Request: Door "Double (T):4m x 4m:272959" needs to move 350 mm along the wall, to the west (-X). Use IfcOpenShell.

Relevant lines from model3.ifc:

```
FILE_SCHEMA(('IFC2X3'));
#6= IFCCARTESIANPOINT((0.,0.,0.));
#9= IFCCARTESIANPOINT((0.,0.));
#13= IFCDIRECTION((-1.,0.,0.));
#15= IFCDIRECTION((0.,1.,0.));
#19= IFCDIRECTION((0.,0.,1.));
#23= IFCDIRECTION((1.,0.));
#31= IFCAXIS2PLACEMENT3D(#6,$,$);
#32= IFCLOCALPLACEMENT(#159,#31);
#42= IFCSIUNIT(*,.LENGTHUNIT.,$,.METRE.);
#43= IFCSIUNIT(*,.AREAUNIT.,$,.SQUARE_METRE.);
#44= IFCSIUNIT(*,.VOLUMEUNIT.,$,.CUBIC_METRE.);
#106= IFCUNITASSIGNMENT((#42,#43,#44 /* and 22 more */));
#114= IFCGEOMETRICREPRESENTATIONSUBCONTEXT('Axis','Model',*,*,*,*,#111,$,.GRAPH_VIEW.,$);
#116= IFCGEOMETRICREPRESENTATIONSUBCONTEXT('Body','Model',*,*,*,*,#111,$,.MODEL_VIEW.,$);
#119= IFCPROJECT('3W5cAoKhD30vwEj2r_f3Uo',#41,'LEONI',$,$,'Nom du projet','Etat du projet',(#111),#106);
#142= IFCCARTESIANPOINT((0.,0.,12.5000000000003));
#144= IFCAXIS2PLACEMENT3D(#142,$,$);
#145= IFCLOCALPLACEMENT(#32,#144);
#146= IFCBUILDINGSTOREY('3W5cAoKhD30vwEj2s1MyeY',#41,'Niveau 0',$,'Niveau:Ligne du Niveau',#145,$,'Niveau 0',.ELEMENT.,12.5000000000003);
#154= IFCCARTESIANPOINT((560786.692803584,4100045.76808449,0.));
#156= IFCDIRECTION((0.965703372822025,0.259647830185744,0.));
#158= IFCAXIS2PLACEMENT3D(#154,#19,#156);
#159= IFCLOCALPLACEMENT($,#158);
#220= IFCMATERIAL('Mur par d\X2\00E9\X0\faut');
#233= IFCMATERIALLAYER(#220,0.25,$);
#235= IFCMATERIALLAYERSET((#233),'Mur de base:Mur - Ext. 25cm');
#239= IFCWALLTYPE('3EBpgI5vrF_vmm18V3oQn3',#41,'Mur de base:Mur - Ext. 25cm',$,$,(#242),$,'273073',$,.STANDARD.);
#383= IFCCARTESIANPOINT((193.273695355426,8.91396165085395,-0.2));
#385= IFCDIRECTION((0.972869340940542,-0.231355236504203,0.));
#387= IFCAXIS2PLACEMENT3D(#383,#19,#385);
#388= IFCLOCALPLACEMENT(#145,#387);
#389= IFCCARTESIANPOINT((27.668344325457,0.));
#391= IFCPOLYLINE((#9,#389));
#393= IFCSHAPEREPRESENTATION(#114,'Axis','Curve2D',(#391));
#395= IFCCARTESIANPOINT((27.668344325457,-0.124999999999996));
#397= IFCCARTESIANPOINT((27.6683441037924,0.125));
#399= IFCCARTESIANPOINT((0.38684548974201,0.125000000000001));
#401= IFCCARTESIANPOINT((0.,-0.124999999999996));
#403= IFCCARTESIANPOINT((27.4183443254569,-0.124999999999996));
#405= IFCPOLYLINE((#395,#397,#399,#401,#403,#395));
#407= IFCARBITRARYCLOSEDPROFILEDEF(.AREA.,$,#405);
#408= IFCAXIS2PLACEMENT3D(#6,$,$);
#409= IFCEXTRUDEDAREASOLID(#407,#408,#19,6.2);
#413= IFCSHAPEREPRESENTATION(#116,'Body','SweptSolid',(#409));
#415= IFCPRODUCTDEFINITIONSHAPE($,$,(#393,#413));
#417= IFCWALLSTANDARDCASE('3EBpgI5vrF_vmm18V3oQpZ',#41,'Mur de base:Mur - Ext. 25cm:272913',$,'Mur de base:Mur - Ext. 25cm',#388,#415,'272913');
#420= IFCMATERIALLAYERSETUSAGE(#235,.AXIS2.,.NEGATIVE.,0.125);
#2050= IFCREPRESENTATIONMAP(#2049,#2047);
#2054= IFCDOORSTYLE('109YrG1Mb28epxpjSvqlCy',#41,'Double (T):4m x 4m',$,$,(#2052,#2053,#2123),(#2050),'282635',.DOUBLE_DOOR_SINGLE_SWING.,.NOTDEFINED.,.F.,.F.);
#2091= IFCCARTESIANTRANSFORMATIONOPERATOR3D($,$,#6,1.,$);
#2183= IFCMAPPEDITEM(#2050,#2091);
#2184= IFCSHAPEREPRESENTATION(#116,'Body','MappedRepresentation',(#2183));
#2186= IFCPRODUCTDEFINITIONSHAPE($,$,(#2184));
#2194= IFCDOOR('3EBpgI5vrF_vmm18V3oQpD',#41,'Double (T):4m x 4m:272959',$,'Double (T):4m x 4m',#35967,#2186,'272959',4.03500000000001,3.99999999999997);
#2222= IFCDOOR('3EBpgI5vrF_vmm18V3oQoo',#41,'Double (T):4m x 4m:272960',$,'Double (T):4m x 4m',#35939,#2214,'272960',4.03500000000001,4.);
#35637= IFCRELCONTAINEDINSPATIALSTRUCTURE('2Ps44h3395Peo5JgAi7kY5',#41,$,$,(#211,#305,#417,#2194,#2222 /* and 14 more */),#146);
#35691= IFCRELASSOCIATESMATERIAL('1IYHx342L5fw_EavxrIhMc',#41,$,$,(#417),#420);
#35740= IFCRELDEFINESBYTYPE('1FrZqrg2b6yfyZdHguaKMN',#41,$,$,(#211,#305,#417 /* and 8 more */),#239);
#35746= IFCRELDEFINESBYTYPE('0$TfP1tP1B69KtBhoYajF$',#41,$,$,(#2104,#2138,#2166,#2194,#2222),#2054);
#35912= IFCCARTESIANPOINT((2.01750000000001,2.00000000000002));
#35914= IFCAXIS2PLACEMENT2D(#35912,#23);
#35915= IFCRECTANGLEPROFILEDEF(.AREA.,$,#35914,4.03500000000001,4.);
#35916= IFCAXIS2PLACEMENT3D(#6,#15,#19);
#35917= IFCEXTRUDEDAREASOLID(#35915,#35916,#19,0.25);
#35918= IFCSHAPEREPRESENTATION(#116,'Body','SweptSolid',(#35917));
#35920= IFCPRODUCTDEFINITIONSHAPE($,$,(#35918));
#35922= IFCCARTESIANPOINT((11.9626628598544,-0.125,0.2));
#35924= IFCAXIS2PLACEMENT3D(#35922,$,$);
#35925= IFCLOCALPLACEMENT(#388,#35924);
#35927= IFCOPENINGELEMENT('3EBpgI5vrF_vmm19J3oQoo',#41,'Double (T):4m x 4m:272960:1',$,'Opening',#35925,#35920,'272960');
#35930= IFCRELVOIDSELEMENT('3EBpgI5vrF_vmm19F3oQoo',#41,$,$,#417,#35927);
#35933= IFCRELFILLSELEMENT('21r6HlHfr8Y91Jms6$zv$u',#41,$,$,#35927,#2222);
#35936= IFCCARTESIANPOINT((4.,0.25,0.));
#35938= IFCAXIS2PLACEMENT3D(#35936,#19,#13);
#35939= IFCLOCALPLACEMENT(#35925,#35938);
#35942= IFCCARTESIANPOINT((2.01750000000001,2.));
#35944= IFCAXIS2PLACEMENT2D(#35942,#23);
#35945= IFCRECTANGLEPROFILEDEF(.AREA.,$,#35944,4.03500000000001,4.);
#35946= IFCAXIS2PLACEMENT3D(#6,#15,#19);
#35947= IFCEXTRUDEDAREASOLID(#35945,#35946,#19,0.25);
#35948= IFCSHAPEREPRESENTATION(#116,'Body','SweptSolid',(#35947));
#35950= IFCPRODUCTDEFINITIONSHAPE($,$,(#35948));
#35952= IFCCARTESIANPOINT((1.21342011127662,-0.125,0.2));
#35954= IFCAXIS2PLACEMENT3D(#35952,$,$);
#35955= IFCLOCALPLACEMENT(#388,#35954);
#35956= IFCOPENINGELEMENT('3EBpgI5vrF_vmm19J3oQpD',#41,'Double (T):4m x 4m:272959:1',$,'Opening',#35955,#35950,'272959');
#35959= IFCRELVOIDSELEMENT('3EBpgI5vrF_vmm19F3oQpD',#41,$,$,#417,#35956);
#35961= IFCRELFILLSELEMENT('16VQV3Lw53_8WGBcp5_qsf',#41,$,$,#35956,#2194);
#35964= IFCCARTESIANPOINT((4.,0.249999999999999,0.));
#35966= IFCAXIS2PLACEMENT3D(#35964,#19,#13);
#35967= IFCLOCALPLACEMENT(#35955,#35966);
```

```python
import ifcopenshell
import ifcopenshell.api.geometry
import ifcopenshell.util.placement

model = ifcopenshell.open("model3.ifc")

door = model.by_id(2194)
opening = door.FillsVoids[0].RelatingOpeningElement
wall = opening.VoidsElements[0].RelatingBuildingElement

wall_matrix = ifcopenshell.util.placement.get_local_placement(wall.ObjectPlacement)
shift = wall_matrix[:3, 0] * -0.35
before = ifcopenshell.util.placement.get_local_placement(door.ObjectPlacement)[:3, 3].copy()

# The door is placed relative to its opening, so it follows when the opening moves.
matrix = ifcopenshell.util.placement.get_local_placement(opening.ObjectPlacement)
matrix[:3, 3] += shift
ifcopenshell.api.geometry.edit_object_placement(
    model, product=opening, matrix=matrix, is_si=False, should_transform_children=True
)

after = ifcopenshell.util.placement.get_local_placement(door.ObjectPlacement)[:3, 3]
print("door moved by", (after - before).round(3) + 0.0)

model.write("model3_v2.ifc")
```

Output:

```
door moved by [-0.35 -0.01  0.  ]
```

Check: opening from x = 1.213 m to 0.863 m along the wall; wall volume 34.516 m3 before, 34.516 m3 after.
